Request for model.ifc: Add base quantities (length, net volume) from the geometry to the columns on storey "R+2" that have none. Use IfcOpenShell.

First a look at what the model holds.

```python
import ifcopenshell
import ifcopenshell.util.element
import ifcopenshell.util.unit

model = ifcopenshell.open("model.ifc")
print(model.schema)
for unit_type in ("LENGTHUNIT", "AREAUNIT", "VOLUMEUNIT"):
    print(unit_type, ifcopenshell.util.unit.calculate_unit_scale(model, unit_type))
storey = next(s for s in model.by_type("IfcBuildingStorey") if s.Name == "R+2")
columns = [e for e in ifcopenshell.util.element.get_decomposition(storey) if e.is_a("IfcColumn")]
for e in sorted(columns, key=lambda e: e.id()):
    print(e.id(), e.is_a(), e.Name, list(ifcopenshell.util.element.get_psets(e, qtos_only=True)), sep=" | ")
```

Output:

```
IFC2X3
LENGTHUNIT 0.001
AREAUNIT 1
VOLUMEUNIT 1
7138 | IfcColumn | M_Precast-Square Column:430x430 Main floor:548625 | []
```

```python
import ifcopenshell
import ifcopenshell.api.pset
import ifcopenshell.geom
import ifcopenshell.util.element
import ifcopenshell.util.shape
import ifcopenshell.util.unit

model = ifcopenshell.open("model.ifc")
unit_scale = ifcopenshell.util.unit.calculate_unit_scale(model)
volume_scale = ifcopenshell.util.unit.calculate_unit_scale(model, "VOLUMEUNIT")
settings = ifcopenshell.geom.settings()

storey = next(s for s in model.by_type("IfcBuildingStorey") if s.Name == "R+2")
columns = [e for e in ifcopenshell.util.element.get_decomposition(storey) if e.is_a("IfcColumn")]

for e in sorted(columns, key=lambda e: e.id()):
    if ifcopenshell.util.element.get_psets(e, qtos_only=True, should_inherit=False):
        continue
    # Geometry comes back in metres, in the element's own axes.
    shape = ifcopenshell.geom.create_shape(settings, e)
    values = {
        "Length": ifcopenshell.util.shape.get_z(shape.geometry) / unit_scale,
        "NetVolume": ifcopenshell.util.shape.get_volume(shape.geometry) / volume_scale,
    }
    qto = ifcopenshell.api.pset.add_qto(model, product=e, name="BaseQuantities")
    ifcopenshell.api.pset.edit_qto(model, qto=qto, properties=values)
    print(e.id(), {k: round(v, 3) for k, v in values.items()})

model.write("model-out.ifc")
```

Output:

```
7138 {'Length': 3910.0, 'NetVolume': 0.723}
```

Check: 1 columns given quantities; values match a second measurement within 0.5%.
